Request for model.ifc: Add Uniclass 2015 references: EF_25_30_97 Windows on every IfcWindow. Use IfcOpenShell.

First a look at what the model holds.

```python
import ifcopenshell

model = ifcopenshell.open("model.ifc")
print(model.schema)
print("classifications:", [c.Name for c in model.by_type("IfcClassification")])
for ifc_class in ("IfcDoor", "IfcRoof", "IfcStair", "IfcWall", "IfcWindow"):
    print(ifc_class, len(model.by_type(ifc_class)))
```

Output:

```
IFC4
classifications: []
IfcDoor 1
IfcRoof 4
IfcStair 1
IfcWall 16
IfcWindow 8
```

```python
import ifcopenshell
import ifcopenshell.api.classification

model = ifcopenshell.open("model.ifc")

system = ifcopenshell.api.classification.add_classification(model, classification="Uniclass 2015")

codes = {
    "IfcWindow": ("EF_25_30_97", "Windows"),
}
for ifc_class, (code, name) in codes.items():
    products = model.by_type(ifc_class)
    ifcopenshell.api.classification.add_reference(
        model, products=products, classification=system, identification=code, name=name
    )
    print(code, len(products))

model.write("model_rev.ifc")
```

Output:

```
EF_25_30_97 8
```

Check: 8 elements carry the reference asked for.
